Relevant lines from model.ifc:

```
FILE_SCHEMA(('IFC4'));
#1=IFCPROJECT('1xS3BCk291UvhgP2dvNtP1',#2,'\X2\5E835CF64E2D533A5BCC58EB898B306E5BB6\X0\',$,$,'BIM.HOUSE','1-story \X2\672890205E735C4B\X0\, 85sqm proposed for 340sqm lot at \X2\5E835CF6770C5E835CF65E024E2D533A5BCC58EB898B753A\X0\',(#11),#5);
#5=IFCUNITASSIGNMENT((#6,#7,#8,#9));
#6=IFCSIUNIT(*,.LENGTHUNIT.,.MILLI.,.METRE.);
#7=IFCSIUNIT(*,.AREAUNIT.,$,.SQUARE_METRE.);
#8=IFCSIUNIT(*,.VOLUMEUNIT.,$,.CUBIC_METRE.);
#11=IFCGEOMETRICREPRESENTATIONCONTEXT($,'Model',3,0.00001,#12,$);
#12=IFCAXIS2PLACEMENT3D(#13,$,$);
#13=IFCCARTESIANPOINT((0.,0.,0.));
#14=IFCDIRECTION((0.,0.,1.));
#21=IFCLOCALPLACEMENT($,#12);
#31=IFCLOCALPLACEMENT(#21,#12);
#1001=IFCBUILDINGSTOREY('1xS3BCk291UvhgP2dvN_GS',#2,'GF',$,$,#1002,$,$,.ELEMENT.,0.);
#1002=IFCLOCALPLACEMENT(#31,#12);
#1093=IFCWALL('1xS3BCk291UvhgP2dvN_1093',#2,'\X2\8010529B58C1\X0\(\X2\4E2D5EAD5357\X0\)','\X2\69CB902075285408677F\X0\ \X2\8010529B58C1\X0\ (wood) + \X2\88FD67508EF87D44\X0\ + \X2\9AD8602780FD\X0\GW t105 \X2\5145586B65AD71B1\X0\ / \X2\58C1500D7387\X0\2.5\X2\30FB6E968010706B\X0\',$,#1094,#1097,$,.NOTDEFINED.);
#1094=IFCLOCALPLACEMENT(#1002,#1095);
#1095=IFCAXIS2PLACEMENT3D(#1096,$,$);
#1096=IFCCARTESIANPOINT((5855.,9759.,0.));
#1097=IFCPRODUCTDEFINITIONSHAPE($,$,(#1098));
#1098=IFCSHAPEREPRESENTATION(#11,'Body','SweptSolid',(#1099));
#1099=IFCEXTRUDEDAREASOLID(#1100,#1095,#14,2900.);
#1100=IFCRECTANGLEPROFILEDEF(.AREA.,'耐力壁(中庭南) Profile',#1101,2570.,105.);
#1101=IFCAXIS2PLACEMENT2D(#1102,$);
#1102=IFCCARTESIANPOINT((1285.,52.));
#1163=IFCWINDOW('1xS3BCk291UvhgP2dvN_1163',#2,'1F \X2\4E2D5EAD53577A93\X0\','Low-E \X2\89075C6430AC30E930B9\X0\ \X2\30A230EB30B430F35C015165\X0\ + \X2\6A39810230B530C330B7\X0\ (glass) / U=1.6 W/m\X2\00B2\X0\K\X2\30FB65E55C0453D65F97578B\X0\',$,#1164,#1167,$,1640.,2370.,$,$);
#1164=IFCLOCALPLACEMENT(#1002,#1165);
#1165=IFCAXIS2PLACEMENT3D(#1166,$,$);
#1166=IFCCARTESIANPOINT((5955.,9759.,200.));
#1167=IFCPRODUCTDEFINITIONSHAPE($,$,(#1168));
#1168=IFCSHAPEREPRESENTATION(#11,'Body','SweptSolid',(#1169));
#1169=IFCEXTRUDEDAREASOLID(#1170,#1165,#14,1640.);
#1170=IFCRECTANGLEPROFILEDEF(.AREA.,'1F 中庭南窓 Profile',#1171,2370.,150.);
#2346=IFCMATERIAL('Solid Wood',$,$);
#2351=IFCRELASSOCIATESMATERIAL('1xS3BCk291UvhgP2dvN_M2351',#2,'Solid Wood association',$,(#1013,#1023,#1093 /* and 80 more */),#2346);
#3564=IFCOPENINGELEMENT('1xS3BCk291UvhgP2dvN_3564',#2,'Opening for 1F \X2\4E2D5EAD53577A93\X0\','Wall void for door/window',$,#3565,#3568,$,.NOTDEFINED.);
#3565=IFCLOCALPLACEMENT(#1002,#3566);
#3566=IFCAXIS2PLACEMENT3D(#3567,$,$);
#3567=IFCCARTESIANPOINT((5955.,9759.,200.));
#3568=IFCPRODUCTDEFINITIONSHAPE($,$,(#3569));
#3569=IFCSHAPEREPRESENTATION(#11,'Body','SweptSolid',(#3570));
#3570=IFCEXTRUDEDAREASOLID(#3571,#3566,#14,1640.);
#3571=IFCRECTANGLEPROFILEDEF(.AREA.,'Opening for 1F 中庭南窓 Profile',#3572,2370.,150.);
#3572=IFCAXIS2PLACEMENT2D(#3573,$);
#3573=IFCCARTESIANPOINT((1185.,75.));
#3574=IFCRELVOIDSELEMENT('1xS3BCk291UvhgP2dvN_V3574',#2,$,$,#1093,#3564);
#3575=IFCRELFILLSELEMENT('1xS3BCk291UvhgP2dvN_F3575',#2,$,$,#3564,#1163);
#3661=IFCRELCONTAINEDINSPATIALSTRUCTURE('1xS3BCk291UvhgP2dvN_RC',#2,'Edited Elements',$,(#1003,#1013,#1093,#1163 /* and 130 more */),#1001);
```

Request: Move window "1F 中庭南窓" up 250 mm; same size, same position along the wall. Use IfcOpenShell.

```python
import numpy as np
import ifcopenshell
import ifcopenshell.api.geometry
import ifcopenshell.util.placement
import ifcopenshell.util.unit

model = ifcopenshell.open("model.ifc")
unit_scale = ifcopenshell.util.unit.calculate_unit_scale(model)

window = model.by_guid("1xS3BCk291UvhgP2dvN_1163")
opening = window.FillsVoids[0].RelatingOpeningElement
dz = 0.25 / unit_scale

shift = np.array([0.0, 0.0, dz])
# The window is not placed relative to its opening, so move both.
for product in (opening, window):
    matrix = ifcopenshell.util.placement.get_local_placement(product.ObjectPlacement)
    matrix[:3, 3] += shift
    ifcopenshell.api.geometry.edit_object_placement(model, product=product, matrix=matrix, is_si=False)

print(f"moved by {dz * unit_scale:+.3f} m")

model.write("model_edited.ifc")
```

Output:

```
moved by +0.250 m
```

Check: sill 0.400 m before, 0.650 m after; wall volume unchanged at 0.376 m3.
